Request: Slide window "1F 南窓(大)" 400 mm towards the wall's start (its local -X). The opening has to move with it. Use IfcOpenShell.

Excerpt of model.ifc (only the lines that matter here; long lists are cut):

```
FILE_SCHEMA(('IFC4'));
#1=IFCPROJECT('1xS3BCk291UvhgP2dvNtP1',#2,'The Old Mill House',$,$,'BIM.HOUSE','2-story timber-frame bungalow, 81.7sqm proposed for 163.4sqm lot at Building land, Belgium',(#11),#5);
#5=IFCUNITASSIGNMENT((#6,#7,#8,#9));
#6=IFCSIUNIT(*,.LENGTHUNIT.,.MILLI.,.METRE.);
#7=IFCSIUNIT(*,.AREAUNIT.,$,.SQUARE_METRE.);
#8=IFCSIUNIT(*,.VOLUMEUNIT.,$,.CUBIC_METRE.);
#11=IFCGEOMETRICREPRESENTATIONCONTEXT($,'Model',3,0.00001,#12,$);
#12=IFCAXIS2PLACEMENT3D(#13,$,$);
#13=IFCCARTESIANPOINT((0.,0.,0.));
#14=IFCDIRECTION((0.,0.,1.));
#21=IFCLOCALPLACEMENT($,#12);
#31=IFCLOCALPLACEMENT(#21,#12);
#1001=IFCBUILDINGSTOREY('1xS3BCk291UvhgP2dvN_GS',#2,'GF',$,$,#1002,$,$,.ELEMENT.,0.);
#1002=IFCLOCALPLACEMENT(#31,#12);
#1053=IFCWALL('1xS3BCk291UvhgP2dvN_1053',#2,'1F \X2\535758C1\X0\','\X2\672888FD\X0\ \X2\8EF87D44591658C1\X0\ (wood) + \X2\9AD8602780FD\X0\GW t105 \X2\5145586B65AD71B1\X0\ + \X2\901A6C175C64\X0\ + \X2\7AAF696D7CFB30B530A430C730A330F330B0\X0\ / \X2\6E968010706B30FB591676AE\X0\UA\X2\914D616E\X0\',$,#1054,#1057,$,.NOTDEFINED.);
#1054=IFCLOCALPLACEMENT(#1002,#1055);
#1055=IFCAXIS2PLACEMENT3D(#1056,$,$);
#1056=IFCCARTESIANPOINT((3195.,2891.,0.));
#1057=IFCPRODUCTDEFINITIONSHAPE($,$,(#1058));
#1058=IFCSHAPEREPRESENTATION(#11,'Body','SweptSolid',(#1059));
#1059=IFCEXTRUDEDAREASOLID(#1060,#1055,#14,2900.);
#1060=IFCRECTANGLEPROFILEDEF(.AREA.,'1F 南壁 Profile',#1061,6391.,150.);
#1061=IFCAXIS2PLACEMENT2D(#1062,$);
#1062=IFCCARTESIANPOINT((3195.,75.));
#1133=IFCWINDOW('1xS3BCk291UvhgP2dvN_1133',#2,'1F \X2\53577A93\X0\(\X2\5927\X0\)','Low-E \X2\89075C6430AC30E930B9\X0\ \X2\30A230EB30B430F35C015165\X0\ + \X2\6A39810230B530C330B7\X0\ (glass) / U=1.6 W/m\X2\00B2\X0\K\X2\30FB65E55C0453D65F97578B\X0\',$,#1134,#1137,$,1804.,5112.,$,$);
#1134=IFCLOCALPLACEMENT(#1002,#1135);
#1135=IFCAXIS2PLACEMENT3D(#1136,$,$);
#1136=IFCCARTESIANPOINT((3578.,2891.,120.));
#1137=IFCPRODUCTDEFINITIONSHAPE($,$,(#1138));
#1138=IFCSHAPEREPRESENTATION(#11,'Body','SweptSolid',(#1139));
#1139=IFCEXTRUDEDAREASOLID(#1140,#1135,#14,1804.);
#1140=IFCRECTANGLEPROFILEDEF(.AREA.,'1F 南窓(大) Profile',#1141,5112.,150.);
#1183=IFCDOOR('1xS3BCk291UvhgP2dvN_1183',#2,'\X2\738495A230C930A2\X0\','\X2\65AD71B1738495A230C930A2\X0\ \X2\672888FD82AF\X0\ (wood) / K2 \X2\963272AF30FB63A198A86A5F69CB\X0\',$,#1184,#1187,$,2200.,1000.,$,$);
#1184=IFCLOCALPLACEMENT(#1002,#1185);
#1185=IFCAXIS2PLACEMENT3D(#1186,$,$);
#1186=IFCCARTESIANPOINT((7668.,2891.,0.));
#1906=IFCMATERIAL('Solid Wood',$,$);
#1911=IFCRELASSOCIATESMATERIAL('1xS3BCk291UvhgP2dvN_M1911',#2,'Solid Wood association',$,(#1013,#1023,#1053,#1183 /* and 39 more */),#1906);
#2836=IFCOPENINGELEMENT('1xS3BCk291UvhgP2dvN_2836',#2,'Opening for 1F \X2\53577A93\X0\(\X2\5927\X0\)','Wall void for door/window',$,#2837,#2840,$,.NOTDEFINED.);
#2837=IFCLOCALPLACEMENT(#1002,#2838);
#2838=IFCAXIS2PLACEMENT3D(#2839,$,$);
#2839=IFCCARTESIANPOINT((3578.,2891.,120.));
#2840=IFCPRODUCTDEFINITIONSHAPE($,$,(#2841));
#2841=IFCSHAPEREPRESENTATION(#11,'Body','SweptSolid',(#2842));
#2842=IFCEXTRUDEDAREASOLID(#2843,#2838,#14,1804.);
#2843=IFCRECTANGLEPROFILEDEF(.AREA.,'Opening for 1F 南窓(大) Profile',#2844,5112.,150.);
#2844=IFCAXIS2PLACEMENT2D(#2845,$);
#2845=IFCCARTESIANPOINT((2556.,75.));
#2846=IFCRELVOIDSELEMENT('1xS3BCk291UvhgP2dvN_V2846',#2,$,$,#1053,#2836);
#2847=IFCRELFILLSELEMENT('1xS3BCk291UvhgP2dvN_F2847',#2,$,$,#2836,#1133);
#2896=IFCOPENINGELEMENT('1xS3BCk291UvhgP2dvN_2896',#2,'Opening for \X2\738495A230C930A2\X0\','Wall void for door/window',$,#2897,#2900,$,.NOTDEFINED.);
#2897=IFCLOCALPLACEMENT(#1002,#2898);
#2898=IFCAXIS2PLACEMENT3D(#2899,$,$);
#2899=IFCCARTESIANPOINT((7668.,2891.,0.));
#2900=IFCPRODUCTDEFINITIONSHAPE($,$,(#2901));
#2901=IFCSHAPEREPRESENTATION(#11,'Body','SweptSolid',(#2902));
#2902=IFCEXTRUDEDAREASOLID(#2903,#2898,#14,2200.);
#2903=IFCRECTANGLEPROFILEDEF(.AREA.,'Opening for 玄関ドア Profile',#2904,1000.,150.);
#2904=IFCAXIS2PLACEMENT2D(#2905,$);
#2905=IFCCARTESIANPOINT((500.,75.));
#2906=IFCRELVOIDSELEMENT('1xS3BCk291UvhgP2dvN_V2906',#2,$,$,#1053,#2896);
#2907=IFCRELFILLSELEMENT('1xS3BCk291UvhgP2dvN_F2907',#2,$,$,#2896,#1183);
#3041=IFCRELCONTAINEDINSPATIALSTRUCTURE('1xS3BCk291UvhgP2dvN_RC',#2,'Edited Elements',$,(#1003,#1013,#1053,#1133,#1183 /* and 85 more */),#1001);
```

```python
import ifcopenshell
import ifcopenshell.api.geometry
import ifcopenshell.util.placement

model = ifcopenshell.open("model.ifc")

window = model.by_guid("1xS3BCk291UvhgP2dvN_1133")
opening = window.FillsVoids[0].RelatingOpeningElement
wall = opening.VoidsElements[0].RelatingBuildingElement

wall_matrix = ifcopenshell.util.placement.get_local_placement(wall.ObjectPlacement)
shift = wall_matrix[:3, 0] * -400.0
before = ifcopenshell.util.placement.get_local_placement(window.ObjectPlacement)[:3, 3].copy()

# The window is not placed relative to its opening, so move both.
for product in (opening, window):
    matrix = ifcopenshell.util.placement.get_local_placement(product.ObjectPlacement)
    matrix[:3, 3] += shift
    ifcopenshell.api.geometry.edit_object_placement(model, product=product, matrix=matrix, is_si=False)

after = ifcopenshell.util.placement.get_local_placement(window.ObjectPlacement)[:3, 3]
print("window moved by", (after - before).round(3) + 0.0)

model.write("model_v2.ifc")
```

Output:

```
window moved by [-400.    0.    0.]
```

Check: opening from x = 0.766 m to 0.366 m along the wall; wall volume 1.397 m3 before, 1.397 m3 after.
